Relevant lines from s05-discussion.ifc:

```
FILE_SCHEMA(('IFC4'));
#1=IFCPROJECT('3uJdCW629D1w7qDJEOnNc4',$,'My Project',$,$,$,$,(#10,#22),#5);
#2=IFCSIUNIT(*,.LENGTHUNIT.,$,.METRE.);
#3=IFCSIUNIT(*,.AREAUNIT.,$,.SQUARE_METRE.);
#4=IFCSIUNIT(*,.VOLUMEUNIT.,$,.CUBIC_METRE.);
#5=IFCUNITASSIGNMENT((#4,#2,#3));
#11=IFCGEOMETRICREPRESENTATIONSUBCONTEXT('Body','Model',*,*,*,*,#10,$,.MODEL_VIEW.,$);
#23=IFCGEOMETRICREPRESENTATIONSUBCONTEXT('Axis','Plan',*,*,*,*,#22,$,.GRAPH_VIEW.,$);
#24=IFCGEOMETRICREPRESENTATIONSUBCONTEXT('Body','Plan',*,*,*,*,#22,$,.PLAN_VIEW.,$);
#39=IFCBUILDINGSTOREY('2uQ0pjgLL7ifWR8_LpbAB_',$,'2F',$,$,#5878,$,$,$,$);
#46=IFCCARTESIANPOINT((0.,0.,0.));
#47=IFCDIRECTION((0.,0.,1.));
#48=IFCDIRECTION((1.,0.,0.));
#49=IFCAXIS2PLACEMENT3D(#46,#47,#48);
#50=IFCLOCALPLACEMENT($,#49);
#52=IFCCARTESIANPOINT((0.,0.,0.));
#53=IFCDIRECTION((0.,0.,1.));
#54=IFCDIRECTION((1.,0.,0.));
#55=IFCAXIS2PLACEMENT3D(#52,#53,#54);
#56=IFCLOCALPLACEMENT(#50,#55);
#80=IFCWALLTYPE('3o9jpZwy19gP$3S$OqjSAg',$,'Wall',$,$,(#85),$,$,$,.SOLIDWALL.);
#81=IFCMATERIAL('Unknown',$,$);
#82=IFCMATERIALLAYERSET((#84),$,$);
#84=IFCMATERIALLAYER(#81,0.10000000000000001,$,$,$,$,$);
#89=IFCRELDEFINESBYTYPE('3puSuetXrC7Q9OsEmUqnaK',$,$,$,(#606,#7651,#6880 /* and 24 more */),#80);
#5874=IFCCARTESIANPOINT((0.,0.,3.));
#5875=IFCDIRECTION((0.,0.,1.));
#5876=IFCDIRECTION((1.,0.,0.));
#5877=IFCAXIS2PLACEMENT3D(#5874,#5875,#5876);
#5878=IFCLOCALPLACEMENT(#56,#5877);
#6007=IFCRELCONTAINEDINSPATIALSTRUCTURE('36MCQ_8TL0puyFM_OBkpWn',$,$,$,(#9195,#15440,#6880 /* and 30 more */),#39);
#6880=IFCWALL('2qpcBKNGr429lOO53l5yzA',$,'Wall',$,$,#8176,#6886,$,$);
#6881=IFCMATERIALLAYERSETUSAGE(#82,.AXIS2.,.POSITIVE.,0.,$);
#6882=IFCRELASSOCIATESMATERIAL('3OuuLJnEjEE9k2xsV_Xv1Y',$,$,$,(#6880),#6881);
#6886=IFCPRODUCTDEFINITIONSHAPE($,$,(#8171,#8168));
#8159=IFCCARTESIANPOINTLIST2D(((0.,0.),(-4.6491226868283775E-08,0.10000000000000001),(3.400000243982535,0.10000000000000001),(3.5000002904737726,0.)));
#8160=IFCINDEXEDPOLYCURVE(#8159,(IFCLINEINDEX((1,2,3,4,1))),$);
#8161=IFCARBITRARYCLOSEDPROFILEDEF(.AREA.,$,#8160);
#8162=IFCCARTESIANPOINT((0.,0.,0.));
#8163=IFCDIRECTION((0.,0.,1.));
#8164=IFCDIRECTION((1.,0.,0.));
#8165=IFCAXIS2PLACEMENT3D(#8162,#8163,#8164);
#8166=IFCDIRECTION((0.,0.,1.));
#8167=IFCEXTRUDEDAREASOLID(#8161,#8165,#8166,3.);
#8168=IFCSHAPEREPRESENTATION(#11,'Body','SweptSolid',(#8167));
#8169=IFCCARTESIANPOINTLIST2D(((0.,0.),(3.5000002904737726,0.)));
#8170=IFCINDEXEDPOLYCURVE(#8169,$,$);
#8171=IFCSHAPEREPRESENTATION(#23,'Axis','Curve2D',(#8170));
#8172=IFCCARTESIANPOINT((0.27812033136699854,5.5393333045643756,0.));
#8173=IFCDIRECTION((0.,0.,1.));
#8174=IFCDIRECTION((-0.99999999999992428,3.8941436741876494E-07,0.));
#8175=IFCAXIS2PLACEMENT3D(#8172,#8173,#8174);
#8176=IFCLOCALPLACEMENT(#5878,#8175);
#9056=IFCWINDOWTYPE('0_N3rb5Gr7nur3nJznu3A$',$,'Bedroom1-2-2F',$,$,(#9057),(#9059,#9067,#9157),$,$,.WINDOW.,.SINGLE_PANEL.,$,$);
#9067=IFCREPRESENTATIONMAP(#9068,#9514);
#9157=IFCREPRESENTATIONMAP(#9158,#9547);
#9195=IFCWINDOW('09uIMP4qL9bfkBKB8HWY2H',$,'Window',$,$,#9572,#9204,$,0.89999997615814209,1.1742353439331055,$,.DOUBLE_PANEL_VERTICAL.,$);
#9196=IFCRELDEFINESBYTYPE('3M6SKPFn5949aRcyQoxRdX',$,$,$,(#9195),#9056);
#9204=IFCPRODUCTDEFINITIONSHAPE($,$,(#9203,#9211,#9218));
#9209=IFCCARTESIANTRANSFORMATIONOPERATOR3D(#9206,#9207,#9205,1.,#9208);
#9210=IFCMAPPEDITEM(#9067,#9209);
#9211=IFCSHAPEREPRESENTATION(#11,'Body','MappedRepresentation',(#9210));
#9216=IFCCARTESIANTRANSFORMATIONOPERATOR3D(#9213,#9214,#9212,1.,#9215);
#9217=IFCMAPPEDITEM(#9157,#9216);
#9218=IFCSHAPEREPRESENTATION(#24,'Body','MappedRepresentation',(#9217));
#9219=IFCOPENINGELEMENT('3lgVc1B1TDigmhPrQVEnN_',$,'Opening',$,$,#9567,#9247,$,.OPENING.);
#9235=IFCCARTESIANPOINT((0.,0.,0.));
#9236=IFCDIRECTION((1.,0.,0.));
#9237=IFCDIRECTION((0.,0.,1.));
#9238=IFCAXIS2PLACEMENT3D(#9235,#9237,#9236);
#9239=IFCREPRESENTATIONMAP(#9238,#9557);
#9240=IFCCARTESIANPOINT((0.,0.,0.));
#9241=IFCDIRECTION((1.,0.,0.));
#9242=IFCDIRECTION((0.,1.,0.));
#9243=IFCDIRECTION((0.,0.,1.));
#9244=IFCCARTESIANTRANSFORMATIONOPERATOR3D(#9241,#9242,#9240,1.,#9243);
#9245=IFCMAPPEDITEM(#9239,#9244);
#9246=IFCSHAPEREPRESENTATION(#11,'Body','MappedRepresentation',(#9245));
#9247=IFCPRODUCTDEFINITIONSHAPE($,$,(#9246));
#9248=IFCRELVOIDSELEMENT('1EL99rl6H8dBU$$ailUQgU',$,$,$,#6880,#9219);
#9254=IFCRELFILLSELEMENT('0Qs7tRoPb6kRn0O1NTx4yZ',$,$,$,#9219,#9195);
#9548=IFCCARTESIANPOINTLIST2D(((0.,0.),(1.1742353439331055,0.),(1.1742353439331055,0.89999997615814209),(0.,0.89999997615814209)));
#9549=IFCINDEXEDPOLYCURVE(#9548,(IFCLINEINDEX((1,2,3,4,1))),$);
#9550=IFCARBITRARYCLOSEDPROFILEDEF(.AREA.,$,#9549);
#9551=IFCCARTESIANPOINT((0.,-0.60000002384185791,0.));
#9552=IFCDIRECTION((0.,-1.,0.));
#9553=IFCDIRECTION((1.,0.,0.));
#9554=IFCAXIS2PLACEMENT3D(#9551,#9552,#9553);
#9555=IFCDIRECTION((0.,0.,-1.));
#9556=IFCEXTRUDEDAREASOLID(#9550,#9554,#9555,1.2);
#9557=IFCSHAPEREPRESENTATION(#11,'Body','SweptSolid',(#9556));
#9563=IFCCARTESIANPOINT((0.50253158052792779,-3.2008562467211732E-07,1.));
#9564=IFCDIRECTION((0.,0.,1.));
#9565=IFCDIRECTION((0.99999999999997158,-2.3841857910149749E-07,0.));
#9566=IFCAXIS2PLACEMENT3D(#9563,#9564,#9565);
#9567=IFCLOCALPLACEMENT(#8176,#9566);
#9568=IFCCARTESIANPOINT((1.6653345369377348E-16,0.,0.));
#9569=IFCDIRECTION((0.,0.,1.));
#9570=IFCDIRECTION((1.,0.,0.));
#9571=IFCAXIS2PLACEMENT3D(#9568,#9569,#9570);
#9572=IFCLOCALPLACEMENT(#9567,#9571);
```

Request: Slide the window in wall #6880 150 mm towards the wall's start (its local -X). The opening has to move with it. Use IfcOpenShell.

```python
import ifcopenshell
import ifcopenshell.api.geometry
import ifcopenshell.util.placement
import ifcopenshell.util.unit

model = ifcopenshell.open("s05-discussion.ifc")
unit_scale = ifcopenshell.util.unit.calculate_unit_scale(model)

window = model.by_guid("09uIMP4qL9bfkBKB8HWY2H")
opening = window.FillsVoids[0].RelatingOpeningElement
wall = opening.VoidsElements[0].RelatingBuildingElement

wall_matrix = ifcopenshell.util.placement.get_local_placement(wall.ObjectPlacement)
shift = wall_matrix[:3, 0] * -0.15 / unit_scale
before = ifcopenshell.util.placement.get_local_placement(window.ObjectPlacement)[:3, 3].copy()

# The window is placed relative to its opening, so it follows when the opening moves.
matrix = ifcopenshell.util.placement.get_local_placement(opening.ObjectPlacement)
matrix[:3, 3] += shift
ifcopenshell.api.geometry.edit_object_placement(
    model, product=opening, matrix=matrix, is_si=False, should_transform_children=True
)

after = ifcopenshell.util.placement.get_local_placement(window.ObjectPlacement)[:3, 3]
print("window moved by", (after - before).round(3) + 0.0)

model.write("s05-discussion_v2.ifc")
```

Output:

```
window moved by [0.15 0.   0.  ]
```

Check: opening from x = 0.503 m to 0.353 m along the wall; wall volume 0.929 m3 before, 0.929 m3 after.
